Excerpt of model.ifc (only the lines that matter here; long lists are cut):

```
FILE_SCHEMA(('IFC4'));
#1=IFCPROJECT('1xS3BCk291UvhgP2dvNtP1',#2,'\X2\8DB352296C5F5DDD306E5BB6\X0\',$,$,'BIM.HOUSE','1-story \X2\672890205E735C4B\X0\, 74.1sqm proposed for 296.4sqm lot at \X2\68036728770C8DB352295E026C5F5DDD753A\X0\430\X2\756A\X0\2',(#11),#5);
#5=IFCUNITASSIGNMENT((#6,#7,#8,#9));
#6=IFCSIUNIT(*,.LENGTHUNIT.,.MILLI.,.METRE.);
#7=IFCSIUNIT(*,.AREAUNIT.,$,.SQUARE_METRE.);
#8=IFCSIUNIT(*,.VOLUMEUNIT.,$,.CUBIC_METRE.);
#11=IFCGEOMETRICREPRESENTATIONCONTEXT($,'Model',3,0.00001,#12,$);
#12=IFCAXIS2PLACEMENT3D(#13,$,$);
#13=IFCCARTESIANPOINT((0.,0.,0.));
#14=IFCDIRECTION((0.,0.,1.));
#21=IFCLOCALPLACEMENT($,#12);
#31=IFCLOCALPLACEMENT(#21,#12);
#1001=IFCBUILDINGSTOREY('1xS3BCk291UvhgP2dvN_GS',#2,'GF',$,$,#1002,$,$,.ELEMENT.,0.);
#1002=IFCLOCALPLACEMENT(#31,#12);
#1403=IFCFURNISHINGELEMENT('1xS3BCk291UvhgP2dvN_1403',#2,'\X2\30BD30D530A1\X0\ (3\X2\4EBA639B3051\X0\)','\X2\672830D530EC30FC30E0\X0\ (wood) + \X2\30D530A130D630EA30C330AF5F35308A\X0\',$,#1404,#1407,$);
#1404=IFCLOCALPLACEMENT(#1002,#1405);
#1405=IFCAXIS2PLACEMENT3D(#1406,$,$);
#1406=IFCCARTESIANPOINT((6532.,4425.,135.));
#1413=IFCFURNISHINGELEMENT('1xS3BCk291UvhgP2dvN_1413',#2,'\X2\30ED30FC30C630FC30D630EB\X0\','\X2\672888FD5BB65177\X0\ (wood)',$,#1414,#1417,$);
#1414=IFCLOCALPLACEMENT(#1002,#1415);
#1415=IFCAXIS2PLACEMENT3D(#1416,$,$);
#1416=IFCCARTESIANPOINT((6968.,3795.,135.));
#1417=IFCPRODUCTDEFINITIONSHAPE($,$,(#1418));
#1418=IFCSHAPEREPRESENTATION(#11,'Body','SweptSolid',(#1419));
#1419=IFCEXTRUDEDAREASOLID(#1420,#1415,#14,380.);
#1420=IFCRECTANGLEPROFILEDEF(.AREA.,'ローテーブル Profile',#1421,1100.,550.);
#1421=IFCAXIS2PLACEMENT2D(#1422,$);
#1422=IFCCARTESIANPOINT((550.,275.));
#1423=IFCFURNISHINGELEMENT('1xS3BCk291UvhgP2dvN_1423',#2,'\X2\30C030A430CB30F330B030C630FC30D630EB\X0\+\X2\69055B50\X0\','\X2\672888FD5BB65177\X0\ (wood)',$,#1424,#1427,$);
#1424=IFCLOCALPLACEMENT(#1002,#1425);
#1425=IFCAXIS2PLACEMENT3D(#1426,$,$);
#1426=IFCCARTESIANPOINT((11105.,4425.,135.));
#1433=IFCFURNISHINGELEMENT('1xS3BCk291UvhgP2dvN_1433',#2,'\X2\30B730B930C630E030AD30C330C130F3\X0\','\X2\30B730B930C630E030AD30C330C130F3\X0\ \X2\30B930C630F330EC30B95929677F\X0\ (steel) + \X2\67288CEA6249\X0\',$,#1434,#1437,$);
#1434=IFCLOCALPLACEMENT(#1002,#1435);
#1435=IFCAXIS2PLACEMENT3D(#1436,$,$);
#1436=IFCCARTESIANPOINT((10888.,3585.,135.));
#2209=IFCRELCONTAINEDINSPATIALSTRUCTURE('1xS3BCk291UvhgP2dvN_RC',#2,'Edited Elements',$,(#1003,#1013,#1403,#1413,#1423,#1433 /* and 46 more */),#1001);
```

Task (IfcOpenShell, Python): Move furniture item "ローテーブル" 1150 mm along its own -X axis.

```python
import ifcopenshell
import ifcopenshell.api.geometry
import ifcopenshell.util.placement
import ifcopenshell.util.unit

model = ifcopenshell.open("model.ifc")
unit_scale = ifcopenshell.util.unit.calculate_unit_scale(model)

item = model.by_guid("1xS3BCk291UvhgP2dvN_1413")
matrix = ifcopenshell.util.placement.get_local_placement(item.ObjectPlacement)
matrix[:3, 3] -= matrix[:3, 0] * 1.15 / unit_scale
ifcopenshell.api.geometry.edit_object_placement(model, product=item, matrix=matrix, is_si=False)

print(ifcopenshell.util.placement.get_local_placement(item.ObjectPlacement).round(3) + 0.0)

model.write("model_v2.ifc")
```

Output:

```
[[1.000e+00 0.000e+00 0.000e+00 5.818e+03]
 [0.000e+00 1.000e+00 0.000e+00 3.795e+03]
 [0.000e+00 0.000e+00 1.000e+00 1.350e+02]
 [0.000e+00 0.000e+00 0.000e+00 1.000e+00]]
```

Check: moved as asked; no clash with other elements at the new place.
